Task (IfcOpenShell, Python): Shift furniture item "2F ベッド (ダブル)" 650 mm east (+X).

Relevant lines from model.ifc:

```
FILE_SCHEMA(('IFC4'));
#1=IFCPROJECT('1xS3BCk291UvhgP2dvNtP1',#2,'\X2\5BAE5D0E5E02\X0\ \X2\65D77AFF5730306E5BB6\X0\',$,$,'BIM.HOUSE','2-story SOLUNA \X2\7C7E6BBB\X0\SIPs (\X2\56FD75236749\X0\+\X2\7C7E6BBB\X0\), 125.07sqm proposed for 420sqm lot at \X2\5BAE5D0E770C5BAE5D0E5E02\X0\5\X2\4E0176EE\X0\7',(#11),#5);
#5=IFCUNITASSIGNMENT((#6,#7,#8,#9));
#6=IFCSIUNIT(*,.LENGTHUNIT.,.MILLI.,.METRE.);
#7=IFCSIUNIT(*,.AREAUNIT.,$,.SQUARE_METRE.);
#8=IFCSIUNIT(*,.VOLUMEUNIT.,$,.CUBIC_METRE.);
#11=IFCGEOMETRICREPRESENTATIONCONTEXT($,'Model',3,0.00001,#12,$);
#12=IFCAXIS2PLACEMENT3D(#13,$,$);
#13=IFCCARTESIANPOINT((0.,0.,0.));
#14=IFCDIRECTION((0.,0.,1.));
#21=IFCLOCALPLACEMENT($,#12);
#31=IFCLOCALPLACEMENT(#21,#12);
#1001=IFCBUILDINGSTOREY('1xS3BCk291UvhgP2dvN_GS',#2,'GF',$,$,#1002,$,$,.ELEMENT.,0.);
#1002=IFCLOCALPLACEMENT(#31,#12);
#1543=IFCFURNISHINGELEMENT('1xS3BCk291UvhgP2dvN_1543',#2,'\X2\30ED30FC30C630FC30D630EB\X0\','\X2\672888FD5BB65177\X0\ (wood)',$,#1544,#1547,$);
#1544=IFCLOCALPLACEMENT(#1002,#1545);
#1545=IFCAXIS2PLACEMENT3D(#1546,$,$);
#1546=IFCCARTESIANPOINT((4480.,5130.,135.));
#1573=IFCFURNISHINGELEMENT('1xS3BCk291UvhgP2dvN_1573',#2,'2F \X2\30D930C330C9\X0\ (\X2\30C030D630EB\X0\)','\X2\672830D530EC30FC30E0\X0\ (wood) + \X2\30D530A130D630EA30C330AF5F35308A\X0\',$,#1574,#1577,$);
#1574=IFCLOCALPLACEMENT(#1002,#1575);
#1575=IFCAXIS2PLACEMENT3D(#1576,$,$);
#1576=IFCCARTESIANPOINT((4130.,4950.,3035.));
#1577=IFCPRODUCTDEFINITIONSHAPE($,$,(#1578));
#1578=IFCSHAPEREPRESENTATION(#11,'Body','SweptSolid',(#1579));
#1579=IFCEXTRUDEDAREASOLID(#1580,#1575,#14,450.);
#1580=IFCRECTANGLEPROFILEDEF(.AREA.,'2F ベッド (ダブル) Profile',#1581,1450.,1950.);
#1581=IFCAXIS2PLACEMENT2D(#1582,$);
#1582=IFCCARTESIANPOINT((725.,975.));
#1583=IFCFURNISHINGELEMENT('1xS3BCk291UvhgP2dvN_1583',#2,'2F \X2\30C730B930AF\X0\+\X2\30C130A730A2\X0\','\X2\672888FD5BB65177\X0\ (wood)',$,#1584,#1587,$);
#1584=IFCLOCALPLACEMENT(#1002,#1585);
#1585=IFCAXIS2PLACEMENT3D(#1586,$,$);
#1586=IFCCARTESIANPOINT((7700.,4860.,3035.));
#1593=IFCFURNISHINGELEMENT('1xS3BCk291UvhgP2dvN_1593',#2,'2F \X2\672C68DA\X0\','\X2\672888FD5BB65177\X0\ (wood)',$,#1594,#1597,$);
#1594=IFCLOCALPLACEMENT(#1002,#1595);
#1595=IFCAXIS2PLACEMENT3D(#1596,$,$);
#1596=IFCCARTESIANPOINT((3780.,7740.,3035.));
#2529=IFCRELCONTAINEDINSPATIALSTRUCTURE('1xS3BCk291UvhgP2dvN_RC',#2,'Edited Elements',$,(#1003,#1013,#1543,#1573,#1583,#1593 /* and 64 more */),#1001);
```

```python
import ifcopenshell
import ifcopenshell.api.geometry
import ifcopenshell.util.placement
import ifcopenshell.util.unit

model = ifcopenshell.open("model.ifc")
unit_scale = ifcopenshell.util.unit.calculate_unit_scale(model)

item = model.by_guid("1xS3BCk291UvhgP2dvN_1573")
matrix = ifcopenshell.util.placement.get_local_placement(item.ObjectPlacement)
matrix[0, 3] += 0.65 / unit_scale
ifcopenshell.api.geometry.edit_object_placement(model, product=item, matrix=matrix, is_si=False)

print(ifcopenshell.util.placement.get_local_placement(item.ObjectPlacement).round(3) + 0.0)

model.write("model_v2.ifc")
```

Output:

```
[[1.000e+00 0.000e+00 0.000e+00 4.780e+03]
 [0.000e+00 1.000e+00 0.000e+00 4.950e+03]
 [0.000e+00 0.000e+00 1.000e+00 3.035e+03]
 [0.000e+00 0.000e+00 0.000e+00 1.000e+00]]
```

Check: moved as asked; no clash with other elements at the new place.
